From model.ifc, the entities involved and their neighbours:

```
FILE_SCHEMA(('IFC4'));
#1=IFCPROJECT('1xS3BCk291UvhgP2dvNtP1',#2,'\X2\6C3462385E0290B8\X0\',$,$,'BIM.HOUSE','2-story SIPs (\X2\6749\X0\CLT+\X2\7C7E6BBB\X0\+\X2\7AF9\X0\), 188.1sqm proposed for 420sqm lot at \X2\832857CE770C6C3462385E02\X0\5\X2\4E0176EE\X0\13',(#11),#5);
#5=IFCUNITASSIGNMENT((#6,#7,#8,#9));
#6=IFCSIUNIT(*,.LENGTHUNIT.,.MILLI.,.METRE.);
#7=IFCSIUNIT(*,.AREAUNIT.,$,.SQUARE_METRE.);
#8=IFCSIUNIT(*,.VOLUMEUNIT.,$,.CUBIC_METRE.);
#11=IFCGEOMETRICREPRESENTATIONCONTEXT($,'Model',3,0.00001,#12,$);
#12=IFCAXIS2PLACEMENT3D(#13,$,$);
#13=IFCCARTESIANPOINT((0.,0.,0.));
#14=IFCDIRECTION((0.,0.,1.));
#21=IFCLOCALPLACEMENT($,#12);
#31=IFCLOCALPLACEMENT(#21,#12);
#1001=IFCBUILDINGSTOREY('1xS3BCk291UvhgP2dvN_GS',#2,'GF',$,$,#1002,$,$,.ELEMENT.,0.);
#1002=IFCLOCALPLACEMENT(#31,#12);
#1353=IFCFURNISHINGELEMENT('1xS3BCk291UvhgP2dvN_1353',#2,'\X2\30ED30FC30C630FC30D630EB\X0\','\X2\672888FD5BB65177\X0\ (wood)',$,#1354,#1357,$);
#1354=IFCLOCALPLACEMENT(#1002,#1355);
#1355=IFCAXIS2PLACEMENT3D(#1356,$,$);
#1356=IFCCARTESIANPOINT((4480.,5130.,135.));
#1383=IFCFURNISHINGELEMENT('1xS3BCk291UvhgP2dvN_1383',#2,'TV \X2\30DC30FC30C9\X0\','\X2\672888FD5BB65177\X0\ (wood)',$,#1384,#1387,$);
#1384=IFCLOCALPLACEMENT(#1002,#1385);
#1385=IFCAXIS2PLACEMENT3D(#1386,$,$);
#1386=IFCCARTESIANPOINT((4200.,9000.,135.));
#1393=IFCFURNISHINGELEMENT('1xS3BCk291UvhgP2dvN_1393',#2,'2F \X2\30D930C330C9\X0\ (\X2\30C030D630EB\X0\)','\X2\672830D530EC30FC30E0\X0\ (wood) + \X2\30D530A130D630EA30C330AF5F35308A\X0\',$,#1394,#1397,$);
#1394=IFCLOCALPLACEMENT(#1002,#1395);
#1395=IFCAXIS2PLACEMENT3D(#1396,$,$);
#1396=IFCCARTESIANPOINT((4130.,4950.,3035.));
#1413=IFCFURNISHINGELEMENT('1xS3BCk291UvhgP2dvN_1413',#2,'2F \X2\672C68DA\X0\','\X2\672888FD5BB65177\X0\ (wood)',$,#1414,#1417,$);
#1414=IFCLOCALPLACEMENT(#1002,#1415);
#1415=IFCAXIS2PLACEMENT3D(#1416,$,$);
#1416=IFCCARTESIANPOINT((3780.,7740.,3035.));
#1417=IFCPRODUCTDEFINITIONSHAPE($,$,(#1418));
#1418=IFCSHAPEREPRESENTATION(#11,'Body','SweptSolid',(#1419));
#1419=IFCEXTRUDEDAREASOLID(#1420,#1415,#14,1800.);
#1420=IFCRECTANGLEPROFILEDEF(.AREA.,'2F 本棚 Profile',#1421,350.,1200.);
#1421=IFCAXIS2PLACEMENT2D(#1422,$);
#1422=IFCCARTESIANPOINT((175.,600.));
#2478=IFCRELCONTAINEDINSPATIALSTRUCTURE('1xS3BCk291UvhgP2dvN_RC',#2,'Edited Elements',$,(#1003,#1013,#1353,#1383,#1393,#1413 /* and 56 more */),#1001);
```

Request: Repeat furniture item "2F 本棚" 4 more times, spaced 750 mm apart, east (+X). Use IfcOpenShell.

```python
import numpy as np
import ifcopenshell
import ifcopenshell.api.geometry
import ifcopenshell.api.root
import ifcopenshell.util.element
import ifcopenshell.util.placement
import ifcopenshell.util.unit

model = ifcopenshell.open("model.ifc")
unit_scale = ifcopenshell.util.unit.calculate_unit_scale(model)


def reuse_history(source, copy):
    """copy_class also copies each property set's owner history, people and application; keep the originals."""
    for rel in copy.IsDefinedBy:
        if rel.is_a("IfcRelDefinesByProperties") and (history := rel.RelatingPropertyDefinition.OwnerHistory):
            rel.RelatingPropertyDefinition.OwnerHistory = source.OwnerHistory
            ifcopenshell.util.element.remove_deep2(model, history)


source = model.by_guid("1xS3BCk291UvhgP2dvN_1413")
base = ifcopenshell.util.placement.get_local_placement(source.ObjectPlacement)
step = np.array([1.0, 0.0, 0.0]) * 0.75 / unit_scale

for i in range(1, 5):
    copy = ifcopenshell.api.root.copy_class(model, product=source)
    copy.Representation = ifcopenshell.util.element.copy_deep(
        model, source.Representation, exclude=["IfcGeometricRepresentationContext", "IfcRepresentationMap"]
    )
    reuse_history(source, copy)
    matrix = base.copy()
    matrix[:3, 3] += i * step
    print("added at", matrix[:3, 3].round(3) + 0.0)
    ifcopenshell.api.geometry.edit_object_placement(model, product=copy, matrix=matrix, is_si=False)

model.write("model_edited.ifc")
```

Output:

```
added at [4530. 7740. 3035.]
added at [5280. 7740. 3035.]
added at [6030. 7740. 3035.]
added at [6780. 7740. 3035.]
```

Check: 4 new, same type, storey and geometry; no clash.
